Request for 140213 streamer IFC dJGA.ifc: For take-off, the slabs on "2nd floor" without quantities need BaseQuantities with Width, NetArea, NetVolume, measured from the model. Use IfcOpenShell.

First a look at what the model holds.

```python
import ifcopenshell
import ifcopenshell.util.element
import ifcopenshell.util.unit

model = ifcopenshell.open("140213 streamer IFC dJGA.ifc")
print(model.schema)
for unit_type in ("LENGTHUNIT", "AREAUNIT", "VOLUMEUNIT"):
    print(unit_type, ifcopenshell.util.unit.calculate_unit_scale(model, unit_type))
storey = next(s for s in model.by_type("IfcBuildingStorey") if s.Name == "2nd floor")
slabs = [e for e in ifcopenshell.util.element.get_decomposition(storey) if e.is_a("IfcSlab")]
for e in sorted(slabs, key=lambda e: e.id()):
    print(e.id(), e.is_a(), e.Name, list(ifcopenshell.util.element.get_psets(e, qtos_only=True)), sep=" | ")
```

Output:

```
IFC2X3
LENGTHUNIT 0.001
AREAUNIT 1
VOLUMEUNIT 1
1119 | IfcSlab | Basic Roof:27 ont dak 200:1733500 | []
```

```python
import ifcopenshell
import ifcopenshell.api.pset
import ifcopenshell.geom
import ifcopenshell.util.element
import ifcopenshell.util.shape
import ifcopenshell.util.unit

model = ifcopenshell.open("140213 streamer IFC dJGA.ifc")
unit_scale = ifcopenshell.util.unit.calculate_unit_scale(model)
area_scale = ifcopenshell.util.unit.calculate_unit_scale(model, "AREAUNIT")
volume_scale = ifcopenshell.util.unit.calculate_unit_scale(model, "VOLUMEUNIT")
settings = ifcopenshell.geom.settings()

storey = next(s for s in model.by_type("IfcBuildingStorey") if s.Name == "2nd floor")
slabs = [e for e in ifcopenshell.util.element.get_decomposition(storey) if e.is_a("IfcSlab")]

for e in sorted(slabs, key=lambda e: e.id()):
    if ifcopenshell.util.element.get_psets(e, qtos_only=True, should_inherit=False):
        continue
    # Geometry comes back in metres, in the element's own axes.
    shape = ifcopenshell.geom.create_shape(settings, e)
    values = {
        "Width": ifcopenshell.util.shape.get_z(shape.geometry) / unit_scale,
        "NetArea": ifcopenshell.util.shape.get_footprint_area(shape.geometry) / area_scale,
        "NetVolume": ifcopenshell.util.shape.get_volume(shape.geometry) / volume_scale,
    }
    qto = ifcopenshell.api.pset.add_qto(model, product=e, name="BaseQuantities")
    ifcopenshell.api.pset.edit_qto(model, qto=qto, properties=values)
    print(e.id(), {k: round(v, 3) for k, v in values.items()})

model.write("140213 streamer IFC dJGA_edited.ifc")
```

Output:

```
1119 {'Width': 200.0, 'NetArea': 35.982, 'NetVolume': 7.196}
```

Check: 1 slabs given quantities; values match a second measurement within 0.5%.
